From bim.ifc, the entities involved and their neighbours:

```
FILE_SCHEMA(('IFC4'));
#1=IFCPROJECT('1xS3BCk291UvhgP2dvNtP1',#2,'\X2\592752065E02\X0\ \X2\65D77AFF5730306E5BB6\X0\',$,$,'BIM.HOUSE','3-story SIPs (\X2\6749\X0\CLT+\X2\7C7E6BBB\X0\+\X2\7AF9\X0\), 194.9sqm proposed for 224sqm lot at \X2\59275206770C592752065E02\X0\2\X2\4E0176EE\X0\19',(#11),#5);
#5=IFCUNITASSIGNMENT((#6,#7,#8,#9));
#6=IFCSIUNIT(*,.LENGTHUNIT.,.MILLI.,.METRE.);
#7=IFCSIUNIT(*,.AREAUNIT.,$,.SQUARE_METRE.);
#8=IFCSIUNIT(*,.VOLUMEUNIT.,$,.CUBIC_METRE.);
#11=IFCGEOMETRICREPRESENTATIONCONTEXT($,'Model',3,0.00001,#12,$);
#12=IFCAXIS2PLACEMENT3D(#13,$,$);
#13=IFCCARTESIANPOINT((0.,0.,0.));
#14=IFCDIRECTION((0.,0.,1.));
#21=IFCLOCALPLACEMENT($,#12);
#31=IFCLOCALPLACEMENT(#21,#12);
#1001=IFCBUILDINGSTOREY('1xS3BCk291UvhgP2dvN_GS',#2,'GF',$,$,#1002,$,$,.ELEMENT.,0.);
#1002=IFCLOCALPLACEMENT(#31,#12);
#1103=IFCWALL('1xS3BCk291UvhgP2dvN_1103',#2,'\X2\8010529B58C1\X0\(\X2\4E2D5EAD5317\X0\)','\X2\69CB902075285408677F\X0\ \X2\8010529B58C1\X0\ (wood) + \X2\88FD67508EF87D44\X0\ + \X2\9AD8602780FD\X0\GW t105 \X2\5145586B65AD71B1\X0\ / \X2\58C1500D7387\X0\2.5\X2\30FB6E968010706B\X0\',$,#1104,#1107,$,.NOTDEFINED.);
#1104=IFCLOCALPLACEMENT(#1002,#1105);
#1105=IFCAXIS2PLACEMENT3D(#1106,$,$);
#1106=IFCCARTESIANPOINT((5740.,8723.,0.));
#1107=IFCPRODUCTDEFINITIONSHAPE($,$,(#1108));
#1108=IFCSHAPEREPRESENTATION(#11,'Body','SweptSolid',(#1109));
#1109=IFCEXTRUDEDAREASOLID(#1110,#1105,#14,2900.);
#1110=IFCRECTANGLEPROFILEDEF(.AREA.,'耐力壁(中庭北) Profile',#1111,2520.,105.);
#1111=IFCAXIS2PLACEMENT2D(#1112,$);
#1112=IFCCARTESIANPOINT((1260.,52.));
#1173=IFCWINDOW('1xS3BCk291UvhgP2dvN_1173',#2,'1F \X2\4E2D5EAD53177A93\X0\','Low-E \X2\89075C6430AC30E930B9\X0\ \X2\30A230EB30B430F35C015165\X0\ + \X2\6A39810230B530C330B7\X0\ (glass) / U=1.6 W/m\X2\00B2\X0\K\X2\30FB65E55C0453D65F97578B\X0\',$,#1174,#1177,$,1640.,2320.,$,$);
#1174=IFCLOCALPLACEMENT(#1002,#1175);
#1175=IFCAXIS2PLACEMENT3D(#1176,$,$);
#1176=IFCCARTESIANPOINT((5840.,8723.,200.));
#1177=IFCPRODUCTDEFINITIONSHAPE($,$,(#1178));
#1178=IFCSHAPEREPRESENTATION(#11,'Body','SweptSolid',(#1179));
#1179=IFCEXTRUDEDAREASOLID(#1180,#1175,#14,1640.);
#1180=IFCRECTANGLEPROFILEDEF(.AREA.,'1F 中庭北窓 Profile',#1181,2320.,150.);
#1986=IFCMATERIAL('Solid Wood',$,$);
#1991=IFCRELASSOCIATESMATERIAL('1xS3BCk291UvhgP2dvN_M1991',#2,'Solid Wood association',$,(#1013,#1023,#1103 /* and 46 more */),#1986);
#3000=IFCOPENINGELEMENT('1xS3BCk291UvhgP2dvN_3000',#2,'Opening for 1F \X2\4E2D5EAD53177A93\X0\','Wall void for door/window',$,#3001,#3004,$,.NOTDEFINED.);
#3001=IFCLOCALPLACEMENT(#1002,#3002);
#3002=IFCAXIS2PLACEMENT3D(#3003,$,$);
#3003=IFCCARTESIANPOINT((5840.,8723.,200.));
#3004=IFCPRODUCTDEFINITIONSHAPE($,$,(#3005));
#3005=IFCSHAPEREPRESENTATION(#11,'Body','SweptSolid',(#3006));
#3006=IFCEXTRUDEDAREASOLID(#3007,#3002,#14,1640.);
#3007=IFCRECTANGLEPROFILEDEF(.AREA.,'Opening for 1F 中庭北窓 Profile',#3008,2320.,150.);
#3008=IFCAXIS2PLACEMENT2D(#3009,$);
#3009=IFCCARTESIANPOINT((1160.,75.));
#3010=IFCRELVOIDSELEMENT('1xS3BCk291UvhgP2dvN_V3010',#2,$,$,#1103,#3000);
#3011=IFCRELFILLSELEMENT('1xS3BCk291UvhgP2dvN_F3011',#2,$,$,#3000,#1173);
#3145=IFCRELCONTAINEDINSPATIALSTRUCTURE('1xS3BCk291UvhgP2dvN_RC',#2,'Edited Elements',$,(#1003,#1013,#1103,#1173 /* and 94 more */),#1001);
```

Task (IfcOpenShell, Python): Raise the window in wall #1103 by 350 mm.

```python
import numpy as np
import ifcopenshell
import ifcopenshell.api.geometry
import ifcopenshell.util.placement
import ifcopenshell.util.unit

model = ifcopenshell.open("bim.ifc")
unit_scale = ifcopenshell.util.unit.calculate_unit_scale(model)

window = model.by_guid("1xS3BCk291UvhgP2dvN_1173")
opening = window.FillsVoids[0].RelatingOpeningElement
dz = 350.0

shift = np.array([0.0, 0.0, dz])
# The window is not placed relative to its opening, so move both.
for product in (opening, window):
    matrix = ifcopenshell.util.placement.get_local_placement(product.ObjectPlacement)
    matrix[:3, 3] += shift
    ifcopenshell.api.geometry.edit_object_placement(model, product=product, matrix=matrix, is_si=False)

print(f"moved by {dz * unit_scale:+.3f} m")

model.write("bim_updated.ifc")
```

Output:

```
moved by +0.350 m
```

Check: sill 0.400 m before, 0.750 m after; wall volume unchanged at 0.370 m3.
